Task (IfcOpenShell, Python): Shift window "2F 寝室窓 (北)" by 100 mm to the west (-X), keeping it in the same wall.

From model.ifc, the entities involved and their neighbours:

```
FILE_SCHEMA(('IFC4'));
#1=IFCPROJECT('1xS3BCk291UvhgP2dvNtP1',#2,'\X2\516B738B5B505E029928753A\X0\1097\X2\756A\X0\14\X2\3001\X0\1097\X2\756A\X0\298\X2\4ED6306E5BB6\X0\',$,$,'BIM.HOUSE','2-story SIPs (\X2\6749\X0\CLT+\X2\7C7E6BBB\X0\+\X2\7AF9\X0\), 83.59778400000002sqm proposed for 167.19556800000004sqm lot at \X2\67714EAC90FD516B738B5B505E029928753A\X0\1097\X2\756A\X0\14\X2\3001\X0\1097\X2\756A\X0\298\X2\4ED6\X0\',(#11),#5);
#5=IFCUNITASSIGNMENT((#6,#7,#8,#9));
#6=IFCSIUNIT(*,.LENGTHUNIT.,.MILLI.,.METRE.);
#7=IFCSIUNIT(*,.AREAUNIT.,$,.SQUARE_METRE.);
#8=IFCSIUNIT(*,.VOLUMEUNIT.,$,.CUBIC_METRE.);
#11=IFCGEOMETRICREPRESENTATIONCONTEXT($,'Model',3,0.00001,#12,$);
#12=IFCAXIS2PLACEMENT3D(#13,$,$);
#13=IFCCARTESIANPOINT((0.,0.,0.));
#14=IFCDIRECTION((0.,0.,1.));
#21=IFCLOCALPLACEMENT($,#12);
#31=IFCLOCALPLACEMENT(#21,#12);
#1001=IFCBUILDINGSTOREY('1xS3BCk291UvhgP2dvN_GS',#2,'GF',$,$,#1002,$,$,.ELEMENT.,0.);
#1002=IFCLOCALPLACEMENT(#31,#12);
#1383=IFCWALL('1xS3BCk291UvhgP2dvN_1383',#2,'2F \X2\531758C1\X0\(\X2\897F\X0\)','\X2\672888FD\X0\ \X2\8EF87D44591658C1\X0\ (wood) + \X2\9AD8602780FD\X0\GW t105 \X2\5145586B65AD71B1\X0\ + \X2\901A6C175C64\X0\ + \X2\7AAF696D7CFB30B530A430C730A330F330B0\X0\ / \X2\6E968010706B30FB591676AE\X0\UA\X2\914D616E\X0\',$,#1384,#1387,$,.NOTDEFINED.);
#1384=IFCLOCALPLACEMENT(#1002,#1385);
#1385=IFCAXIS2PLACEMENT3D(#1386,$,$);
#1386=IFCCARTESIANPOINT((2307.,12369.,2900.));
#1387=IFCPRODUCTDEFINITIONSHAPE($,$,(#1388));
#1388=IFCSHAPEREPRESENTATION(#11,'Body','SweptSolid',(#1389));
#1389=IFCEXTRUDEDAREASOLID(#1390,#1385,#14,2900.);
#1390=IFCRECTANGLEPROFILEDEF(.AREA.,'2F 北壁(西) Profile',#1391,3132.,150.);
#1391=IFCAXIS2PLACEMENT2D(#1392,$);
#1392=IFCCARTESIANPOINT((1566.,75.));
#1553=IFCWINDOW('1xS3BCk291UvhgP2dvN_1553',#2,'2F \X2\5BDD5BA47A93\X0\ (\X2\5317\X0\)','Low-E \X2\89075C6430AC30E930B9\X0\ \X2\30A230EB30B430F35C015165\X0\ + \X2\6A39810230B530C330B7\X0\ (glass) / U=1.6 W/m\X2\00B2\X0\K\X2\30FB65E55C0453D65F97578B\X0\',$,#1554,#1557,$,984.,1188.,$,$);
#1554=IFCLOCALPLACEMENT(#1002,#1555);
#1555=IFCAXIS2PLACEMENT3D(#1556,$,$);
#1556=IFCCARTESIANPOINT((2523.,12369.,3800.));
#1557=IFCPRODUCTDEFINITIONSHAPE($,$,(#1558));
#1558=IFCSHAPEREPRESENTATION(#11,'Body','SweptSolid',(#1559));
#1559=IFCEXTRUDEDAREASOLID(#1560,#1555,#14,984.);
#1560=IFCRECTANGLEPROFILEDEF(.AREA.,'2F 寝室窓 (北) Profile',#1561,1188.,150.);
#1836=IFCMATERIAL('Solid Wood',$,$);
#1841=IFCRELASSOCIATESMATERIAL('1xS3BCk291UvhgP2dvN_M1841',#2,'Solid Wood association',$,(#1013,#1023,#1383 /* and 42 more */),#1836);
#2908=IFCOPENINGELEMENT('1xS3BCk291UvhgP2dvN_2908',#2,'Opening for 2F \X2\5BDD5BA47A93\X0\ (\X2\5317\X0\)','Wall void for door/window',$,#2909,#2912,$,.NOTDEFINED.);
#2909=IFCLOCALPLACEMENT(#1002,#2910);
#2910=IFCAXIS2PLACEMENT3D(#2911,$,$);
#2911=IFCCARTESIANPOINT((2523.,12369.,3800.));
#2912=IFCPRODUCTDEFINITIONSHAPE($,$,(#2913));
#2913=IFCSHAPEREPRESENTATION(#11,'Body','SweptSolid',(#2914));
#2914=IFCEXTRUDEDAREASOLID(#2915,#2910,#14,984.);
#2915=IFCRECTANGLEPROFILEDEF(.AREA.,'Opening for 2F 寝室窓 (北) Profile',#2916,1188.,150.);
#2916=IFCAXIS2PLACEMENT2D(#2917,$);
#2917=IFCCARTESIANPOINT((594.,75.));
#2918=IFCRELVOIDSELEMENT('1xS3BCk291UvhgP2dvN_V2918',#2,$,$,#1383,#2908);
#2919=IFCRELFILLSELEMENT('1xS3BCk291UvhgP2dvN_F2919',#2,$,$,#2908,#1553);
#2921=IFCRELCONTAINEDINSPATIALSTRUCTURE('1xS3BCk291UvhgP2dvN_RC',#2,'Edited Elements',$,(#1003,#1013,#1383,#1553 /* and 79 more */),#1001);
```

```python
import ifcopenshell
import ifcopenshell.api.geometry
import ifcopenshell.util.placement

model = ifcopenshell.open("model.ifc")

window = model.by_id(1553)
opening = window.FillsVoids[0].RelatingOpeningElement
wall = opening.VoidsElements[0].RelatingBuildingElement

wall_matrix = ifcopenshell.util.placement.get_local_placement(wall.ObjectPlacement)
shift = wall_matrix[:3, 0] * -100.0
before = ifcopenshell.util.placement.get_local_placement(window.ObjectPlacement)[:3, 3].copy()

# The window is not placed relative to its opening, so move both.
for product in (opening, window):
    matrix = ifcopenshell.util.placement.get_local_placement(product.ObjectPlacement)
    matrix[:3, 3] += shift
    ifcopenshell.api.geometry.edit_object_placement(model, product=product, matrix=matrix, is_si=False)

after = ifcopenshell.util.placement.get_local_placement(window.ObjectPlacement)[:3, 3]
print("window moved by", (after - before).round(3) + 0.0)

model.write("model_updated.ifc")
```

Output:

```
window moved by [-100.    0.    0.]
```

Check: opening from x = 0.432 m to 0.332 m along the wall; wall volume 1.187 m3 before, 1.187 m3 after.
